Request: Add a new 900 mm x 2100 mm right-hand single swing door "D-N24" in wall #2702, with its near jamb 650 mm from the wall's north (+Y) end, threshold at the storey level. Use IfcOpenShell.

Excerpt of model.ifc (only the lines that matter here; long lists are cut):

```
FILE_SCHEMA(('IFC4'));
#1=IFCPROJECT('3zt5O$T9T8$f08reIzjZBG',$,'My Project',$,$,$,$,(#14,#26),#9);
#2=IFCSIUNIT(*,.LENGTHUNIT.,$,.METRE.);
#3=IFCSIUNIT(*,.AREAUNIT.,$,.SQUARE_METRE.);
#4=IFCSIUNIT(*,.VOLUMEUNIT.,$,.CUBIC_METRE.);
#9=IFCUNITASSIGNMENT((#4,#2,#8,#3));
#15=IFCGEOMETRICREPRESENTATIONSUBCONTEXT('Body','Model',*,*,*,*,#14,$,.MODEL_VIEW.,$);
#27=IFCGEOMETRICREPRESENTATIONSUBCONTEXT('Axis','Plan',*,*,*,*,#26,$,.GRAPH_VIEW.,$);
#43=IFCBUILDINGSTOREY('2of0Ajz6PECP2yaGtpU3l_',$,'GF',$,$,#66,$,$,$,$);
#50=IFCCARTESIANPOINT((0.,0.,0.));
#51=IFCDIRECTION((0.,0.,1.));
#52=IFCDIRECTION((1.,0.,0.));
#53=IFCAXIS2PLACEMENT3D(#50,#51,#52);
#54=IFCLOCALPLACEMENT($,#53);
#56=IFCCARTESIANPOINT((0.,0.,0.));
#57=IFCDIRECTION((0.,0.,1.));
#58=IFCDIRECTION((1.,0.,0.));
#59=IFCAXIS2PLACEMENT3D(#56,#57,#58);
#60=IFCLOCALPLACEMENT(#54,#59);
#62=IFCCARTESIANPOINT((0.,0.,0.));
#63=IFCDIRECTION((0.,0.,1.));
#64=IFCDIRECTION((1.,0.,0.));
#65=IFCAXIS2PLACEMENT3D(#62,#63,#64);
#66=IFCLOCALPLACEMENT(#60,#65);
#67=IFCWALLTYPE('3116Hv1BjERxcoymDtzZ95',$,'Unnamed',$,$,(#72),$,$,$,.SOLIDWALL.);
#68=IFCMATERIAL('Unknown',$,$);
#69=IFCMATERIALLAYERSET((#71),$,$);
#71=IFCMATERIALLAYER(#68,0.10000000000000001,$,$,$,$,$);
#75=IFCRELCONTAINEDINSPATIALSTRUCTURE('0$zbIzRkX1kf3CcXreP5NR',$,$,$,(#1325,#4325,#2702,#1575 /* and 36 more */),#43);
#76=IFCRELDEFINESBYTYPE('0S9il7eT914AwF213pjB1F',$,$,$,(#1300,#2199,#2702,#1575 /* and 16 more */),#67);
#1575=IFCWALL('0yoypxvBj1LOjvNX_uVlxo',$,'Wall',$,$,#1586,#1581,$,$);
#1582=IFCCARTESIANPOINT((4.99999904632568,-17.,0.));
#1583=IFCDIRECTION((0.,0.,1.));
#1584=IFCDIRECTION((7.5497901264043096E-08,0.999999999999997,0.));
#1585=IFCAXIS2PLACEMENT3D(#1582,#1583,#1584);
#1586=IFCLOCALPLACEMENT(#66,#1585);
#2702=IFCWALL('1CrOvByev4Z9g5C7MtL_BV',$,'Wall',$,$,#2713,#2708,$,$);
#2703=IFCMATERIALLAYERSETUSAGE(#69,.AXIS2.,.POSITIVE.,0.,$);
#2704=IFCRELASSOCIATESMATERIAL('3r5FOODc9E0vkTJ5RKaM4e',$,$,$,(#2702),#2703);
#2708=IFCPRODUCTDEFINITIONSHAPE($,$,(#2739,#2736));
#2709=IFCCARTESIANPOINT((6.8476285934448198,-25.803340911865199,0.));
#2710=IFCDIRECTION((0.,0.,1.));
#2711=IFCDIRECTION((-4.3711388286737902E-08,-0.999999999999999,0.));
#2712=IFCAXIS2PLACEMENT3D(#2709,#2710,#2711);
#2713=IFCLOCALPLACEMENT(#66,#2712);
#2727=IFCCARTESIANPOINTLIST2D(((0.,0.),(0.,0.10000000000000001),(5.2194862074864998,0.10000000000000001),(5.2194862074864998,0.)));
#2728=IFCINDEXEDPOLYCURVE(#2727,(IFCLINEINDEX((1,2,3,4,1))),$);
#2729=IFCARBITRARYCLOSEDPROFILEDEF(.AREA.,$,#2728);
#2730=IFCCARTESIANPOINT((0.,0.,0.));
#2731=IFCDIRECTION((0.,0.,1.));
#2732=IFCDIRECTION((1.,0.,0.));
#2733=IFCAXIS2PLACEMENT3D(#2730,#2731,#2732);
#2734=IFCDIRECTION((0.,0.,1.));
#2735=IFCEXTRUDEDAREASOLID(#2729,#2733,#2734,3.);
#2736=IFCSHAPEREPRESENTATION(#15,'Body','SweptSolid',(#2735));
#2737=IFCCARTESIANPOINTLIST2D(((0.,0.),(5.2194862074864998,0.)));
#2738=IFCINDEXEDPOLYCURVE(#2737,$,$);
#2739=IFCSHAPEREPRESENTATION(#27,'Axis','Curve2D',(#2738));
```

```python
import numpy as np
import ifcopenshell
import ifcopenshell.api.feature
import ifcopenshell.api.geometry
import ifcopenshell.api.root
import ifcopenshell.api.spatial
import ifcopenshell.geom
import ifcopenshell.util.element
import ifcopenshell.util.placement
import ifcopenshell.util.representation
import ifcopenshell.util.shape
import ifcopenshell.util.unit

model = ifcopenshell.open("model.ifc")
unit_scale = ifcopenshell.util.unit.calculate_unit_scale(model)
settings = ifcopenshell.geom.settings()


def volume(element):
    """Net volume in cubic metres, openings subtracted."""
    shape = ifcopenshell.geom.create_shape(settings, element)
    return ifcopenshell.util.shape.get_volume(shape.geometry)


wall = model.by_guid("1CrOvByev4Z9g5C7MtL_BV")
storey = ifcopenshell.util.element.get_container(wall, ifc_class="IfcBuildingStorey")
context = ifcopenshell.util.representation.get_context(model, "Model", "Body", "MODEL_VIEW")
before = volume(wall)

width, height, from_end, sill = 0.9, 2.1, 0.65, 0.0  # metres

# The wall runs along its own X axis, and the end named is its -X end.
wall_shape = ifcopenshell.geom.create_shape(settings, wall)
x, y, z = ifcopenshell.util.shape.get_vertices(wall_shape.geometry).T
start = x.min() + from_end
face, thickness = float(y.min()), float(y.max() - y.min())
wall_matrix = ifcopenshell.util.placement.get_local_placement(wall.ObjectPlacement)
level = ifcopenshell.util.placement.get_local_placement(storey.ObjectPlacement)[2, 3]


def in_wall(x, y):
    """Placement at x, y metres in the wall's axes, at sill height."""
    matrix = wall_matrix.copy()
    matrix[:, 3] = wall_matrix @ np.array([x / unit_scale, y / unit_scale, 0.0, 1.0])
    matrix[2, 3] = level + sill / unit_scale
    return matrix


# Opening: a box that overshoots both wall faces by 50 mm.
opening = ifcopenshell.api.root.create_entity(model, ifc_class="IfcOpeningElement", predefined_type="OPENING")
box = ifcopenshell.api.geometry.add_wall_representation(
    model, context=context, length=width, height=height, thickness=thickness + 0.1
)
ifcopenshell.api.geometry.assign_representation(model, product=opening, representation=box)
ifcopenshell.api.geometry.edit_object_placement(model, product=opening, matrix=in_wall(start, face - 0.05), is_si=False)
ifcopenshell.api.feature.add_feature(model, feature=opening, element=wall)

door = ifcopenshell.api.root.create_entity(model, ifc_class="IfcDoor", name="D-N24", predefined_type="DOOR")
door.OverallWidth, door.OverallHeight = width / unit_scale, height / unit_scale
door.OperationType = "SINGLE_SWING_RIGHT"
body = ifcopenshell.api.geometry.add_door_representation(
    model,
    context=context,
    overall_width=door.OverallWidth,
    overall_height=door.OverallHeight,
    operation_type="SINGLE_SWING_RIGHT",
    lining_properties={"LiningDepth": thickness / unit_scale, "ThresholdDepth": thickness / unit_scale},
)
ifcopenshell.api.geometry.assign_representation(model, product=door, representation=body)
ifcopenshell.api.spatial.assign_container(model, products=[door], relating_structure=storey)
ifcopenshell.api.feature.add_filling(model, opening=opening, element=door)

# The lining spans the wall, so the door starts at the wall face.
ifcopenshell.api.geometry.edit_object_placement(model, product=door, matrix=in_wall(start, face), is_si=False)

after = volume(wall)

print(f"wall volume {before:.3f} -> {after:.3f} m3")

model.write("model_edited.ifc")
```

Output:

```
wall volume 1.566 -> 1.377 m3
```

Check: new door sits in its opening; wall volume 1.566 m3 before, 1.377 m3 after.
